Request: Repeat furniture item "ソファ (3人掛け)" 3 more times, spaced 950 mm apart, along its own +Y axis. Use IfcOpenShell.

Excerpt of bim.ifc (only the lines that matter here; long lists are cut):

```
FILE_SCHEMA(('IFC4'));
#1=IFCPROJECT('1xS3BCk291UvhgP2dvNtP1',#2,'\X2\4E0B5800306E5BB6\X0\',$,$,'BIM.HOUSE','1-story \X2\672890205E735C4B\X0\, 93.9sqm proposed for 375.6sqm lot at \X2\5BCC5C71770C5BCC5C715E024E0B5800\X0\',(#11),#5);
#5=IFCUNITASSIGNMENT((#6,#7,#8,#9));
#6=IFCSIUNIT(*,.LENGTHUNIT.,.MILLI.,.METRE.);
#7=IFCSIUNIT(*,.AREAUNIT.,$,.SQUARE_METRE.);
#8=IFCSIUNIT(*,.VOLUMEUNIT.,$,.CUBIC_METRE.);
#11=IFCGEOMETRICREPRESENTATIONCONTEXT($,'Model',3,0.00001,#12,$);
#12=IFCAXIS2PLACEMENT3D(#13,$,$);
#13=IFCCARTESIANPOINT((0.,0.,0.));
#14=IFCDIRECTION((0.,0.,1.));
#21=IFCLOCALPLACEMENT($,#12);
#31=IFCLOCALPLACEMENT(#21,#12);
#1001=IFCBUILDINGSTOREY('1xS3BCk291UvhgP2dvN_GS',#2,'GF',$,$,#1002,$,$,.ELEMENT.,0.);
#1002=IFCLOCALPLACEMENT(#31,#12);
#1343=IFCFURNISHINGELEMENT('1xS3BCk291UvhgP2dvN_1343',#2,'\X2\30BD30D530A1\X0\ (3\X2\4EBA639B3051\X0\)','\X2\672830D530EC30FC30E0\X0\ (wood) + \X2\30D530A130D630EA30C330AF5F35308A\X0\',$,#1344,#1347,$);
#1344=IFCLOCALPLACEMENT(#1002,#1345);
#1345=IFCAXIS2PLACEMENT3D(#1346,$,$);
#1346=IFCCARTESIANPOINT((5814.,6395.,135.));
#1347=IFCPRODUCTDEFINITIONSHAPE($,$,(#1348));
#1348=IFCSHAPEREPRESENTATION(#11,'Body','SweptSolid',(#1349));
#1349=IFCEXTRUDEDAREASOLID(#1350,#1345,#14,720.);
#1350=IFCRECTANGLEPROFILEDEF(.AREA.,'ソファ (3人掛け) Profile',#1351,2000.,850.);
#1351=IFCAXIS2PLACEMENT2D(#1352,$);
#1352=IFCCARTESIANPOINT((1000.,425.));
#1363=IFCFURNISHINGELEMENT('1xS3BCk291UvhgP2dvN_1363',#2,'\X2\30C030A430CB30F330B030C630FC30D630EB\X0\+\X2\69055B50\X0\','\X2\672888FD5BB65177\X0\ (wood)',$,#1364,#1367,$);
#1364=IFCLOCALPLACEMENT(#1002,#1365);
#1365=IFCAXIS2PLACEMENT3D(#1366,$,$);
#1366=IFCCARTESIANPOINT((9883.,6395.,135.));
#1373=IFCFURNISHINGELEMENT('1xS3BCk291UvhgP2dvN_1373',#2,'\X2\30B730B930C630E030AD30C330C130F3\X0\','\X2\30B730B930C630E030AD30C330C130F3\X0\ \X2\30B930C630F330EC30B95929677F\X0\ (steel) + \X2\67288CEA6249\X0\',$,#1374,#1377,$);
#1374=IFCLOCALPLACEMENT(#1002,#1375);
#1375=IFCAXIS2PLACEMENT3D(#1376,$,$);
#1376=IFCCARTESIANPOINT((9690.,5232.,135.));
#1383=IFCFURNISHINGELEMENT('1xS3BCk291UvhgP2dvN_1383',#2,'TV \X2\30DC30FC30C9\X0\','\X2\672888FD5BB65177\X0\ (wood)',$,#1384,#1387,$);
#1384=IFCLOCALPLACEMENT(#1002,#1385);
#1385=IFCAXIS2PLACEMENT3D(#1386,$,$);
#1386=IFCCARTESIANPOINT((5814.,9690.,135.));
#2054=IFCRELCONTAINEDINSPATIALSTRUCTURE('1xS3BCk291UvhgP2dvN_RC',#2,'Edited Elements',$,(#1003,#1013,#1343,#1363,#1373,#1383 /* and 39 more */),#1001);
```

```python
import ifcopenshell
import ifcopenshell.api.geometry
import ifcopenshell.api.root
import ifcopenshell.util.element
import ifcopenshell.util.placement
import ifcopenshell.util.unit

model = ifcopenshell.open("bim.ifc")
unit_scale = ifcopenshell.util.unit.calculate_unit_scale(model)


def reuse_history(source, copy):
    """copy_class also copies each property set's owner history, people and application; keep the originals."""
    for rel in copy.IsDefinedBy:
        if rel.is_a("IfcRelDefinesByProperties") and (history := rel.RelatingPropertyDefinition.OwnerHistory):
            rel.RelatingPropertyDefinition.OwnerHistory = source.OwnerHistory
            ifcopenshell.util.element.remove_deep2(model, history)


source = model.by_guid("1xS3BCk291UvhgP2dvN_1343")
base = ifcopenshell.util.placement.get_local_placement(source.ObjectPlacement)
step = base[:3, 1] * 0.95 / unit_scale

for i in range(1, 4):
    copy = ifcopenshell.api.root.copy_class(model, product=source)
    copy.Representation = ifcopenshell.util.element.copy_deep(
        model, source.Representation, exclude=["IfcGeometricRepresentationContext", "IfcRepresentationMap"]
    )
    reuse_history(source, copy)
    matrix = base.copy()
    matrix[:3, 3] += i * step
    print("added at", matrix[:3, 3].round(3) + 0.0)
    ifcopenshell.api.geometry.edit_object_placement(model, product=copy, matrix=matrix, is_si=False)

model.write("bim_updated.ifc")
```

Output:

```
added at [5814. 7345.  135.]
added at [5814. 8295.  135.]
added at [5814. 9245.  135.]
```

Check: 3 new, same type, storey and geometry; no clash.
